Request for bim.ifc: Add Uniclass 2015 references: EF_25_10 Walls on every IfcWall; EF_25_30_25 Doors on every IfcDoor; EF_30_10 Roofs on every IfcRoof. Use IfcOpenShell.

First a look at what the model holds.

```python
import ifcopenshell

model = ifcopenshell.open("bim.ifc")
print(model.schema)
print("classifications:", [c.Name for c in model.by_type("IfcClassification")])
for ifc_class in ("IfcDoor", "IfcRoof", "IfcStair", "IfcWall", "IfcWindow"):
    print(ifc_class, len(model.by_type(ifc_class)))
```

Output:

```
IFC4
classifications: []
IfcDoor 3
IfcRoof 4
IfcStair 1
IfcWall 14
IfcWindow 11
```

```python
import ifcopenshell
import ifcopenshell.api.classification

model = ifcopenshell.open("bim.ifc")

system = ifcopenshell.api.classification.add_classification(model, classification="Uniclass 2015")

codes = {
    "IfcWall": ("EF_25_10", "Walls"),
    "IfcDoor": ("EF_25_30_25", "Doors"),
    "IfcRoof": ("EF_30_10", "Roofs"),
}
for ifc_class, (code, name) in codes.items():
    products = model.by_type(ifc_class)
    ifcopenshell.api.classification.add_reference(
        model, products=products, classification=system, identification=code, name=name
    )
    print(code, len(products))

model.write("bim_rev.ifc")
```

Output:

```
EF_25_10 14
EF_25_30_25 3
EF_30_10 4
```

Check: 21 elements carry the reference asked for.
